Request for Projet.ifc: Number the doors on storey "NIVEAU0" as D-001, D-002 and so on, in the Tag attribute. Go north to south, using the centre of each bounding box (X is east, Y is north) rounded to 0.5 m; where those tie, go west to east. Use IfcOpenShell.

First a look at what the model holds.

```python
import ifcopenshell
import ifcopenshell.util.element
import ifcopenshell.util.placement

model = ifcopenshell.open("Projet.ifc")
print(model.schema)
storey = next(s for s in model.by_type("IfcBuildingStorey") if s.Name == "NIVEAU0")
doors = [e for e in ifcopenshell.util.element.get_decomposition(storey) if e.is_a("IfcDoor")]
for e in sorted(doors, key=lambda e: e.id()):
    origin = ifcopenshell.util.placement.get_local_placement(e.ObjectPlacement)[:3, 3]
    print(e.id(), e.Tag, e.Name, origin.round(2) + 0.0, sep=" | ")
```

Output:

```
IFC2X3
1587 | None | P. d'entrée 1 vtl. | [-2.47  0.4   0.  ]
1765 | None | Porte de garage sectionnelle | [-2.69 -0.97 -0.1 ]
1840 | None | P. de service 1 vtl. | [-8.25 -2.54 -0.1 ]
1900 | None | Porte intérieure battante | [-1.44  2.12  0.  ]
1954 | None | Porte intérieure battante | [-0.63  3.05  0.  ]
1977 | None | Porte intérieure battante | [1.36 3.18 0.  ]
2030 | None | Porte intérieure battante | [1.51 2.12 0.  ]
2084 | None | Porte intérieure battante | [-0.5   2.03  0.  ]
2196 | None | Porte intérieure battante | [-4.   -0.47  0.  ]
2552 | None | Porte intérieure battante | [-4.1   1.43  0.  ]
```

```python
import ifcopenshell
import ifcopenshell.geom
import ifcopenshell.util.element
import ifcopenshell.util.shape

model = ifcopenshell.open("Projet.ifc")
settings = ifcopenshell.geom.settings()
settings.set("use-world-coords", True)


def centre(element):
    shape = ifcopenshell.geom.create_shape(settings, element)
    return ifcopenshell.util.shape.get_bbox_centroid(shape.geometry)


storey = next(s for s in model.by_type("IfcBuildingStorey") if s.Name == "NIVEAU0")
doors = [e for e in ifcopenshell.util.element.get_decomposition(storey) if e.is_a("IfcDoor")]

# Insertion points can sit at a corner or the storey origin, so sort by the geometry (in metres).
centres = {e: centre(e) for e in doors}
doors.sort(key=lambda e: (-round(centres[e][1] / 0.5), centres[e][0]))

for i, e in enumerate(doors, start=1):
    number = f"D-0{i:02d}"
    e.Tag = number
    print(e.id(), number)

model.write("Projet-out.ifc")
```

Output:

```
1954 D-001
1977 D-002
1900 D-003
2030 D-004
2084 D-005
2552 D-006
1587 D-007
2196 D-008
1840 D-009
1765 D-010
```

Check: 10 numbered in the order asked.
